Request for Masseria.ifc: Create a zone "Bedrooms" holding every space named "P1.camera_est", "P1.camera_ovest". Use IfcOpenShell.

First a look at what the model holds.

```python
import ifcopenshell

model = ifcopenshell.open("Masseria.ifc")
print(model.schema)
seen = {}
for space in model.by_type("IfcSpace"):
    seen[space.LongName] = seen.get(space.LongName, 0) + 1
for name, count in sorted(seen.items(), key=str):
    print(count, "x", name)
print("zones:", [z.Name for z in model.by_type("IfcZone")][:20])
```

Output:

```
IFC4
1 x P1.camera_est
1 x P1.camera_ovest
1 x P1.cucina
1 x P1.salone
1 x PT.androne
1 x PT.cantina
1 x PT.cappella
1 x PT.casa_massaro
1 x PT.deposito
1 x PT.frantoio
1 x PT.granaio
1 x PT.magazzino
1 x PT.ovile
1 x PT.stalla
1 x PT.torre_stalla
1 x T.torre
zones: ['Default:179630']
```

```python
import ifcopenshell
import ifcopenshell.api.group
import ifcopenshell.api.root

model = ifcopenshell.open("Masseria.ifc")

names = {"P1.camera_est", "P1.camera_ovest"}
spaces = [s for s in model.by_type("IfcSpace") if s.LongName in names]

zone = ifcopenshell.api.root.create_entity(model, ifc_class="IfcZone", name="Bedrooms")
ifcopenshell.api.group.assign_group(model, products=spaces, group=zone)
print(len(spaces), "spaces in", zone.Name)

model.write("Masseria_updated.ifc")
```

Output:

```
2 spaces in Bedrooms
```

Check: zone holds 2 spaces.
